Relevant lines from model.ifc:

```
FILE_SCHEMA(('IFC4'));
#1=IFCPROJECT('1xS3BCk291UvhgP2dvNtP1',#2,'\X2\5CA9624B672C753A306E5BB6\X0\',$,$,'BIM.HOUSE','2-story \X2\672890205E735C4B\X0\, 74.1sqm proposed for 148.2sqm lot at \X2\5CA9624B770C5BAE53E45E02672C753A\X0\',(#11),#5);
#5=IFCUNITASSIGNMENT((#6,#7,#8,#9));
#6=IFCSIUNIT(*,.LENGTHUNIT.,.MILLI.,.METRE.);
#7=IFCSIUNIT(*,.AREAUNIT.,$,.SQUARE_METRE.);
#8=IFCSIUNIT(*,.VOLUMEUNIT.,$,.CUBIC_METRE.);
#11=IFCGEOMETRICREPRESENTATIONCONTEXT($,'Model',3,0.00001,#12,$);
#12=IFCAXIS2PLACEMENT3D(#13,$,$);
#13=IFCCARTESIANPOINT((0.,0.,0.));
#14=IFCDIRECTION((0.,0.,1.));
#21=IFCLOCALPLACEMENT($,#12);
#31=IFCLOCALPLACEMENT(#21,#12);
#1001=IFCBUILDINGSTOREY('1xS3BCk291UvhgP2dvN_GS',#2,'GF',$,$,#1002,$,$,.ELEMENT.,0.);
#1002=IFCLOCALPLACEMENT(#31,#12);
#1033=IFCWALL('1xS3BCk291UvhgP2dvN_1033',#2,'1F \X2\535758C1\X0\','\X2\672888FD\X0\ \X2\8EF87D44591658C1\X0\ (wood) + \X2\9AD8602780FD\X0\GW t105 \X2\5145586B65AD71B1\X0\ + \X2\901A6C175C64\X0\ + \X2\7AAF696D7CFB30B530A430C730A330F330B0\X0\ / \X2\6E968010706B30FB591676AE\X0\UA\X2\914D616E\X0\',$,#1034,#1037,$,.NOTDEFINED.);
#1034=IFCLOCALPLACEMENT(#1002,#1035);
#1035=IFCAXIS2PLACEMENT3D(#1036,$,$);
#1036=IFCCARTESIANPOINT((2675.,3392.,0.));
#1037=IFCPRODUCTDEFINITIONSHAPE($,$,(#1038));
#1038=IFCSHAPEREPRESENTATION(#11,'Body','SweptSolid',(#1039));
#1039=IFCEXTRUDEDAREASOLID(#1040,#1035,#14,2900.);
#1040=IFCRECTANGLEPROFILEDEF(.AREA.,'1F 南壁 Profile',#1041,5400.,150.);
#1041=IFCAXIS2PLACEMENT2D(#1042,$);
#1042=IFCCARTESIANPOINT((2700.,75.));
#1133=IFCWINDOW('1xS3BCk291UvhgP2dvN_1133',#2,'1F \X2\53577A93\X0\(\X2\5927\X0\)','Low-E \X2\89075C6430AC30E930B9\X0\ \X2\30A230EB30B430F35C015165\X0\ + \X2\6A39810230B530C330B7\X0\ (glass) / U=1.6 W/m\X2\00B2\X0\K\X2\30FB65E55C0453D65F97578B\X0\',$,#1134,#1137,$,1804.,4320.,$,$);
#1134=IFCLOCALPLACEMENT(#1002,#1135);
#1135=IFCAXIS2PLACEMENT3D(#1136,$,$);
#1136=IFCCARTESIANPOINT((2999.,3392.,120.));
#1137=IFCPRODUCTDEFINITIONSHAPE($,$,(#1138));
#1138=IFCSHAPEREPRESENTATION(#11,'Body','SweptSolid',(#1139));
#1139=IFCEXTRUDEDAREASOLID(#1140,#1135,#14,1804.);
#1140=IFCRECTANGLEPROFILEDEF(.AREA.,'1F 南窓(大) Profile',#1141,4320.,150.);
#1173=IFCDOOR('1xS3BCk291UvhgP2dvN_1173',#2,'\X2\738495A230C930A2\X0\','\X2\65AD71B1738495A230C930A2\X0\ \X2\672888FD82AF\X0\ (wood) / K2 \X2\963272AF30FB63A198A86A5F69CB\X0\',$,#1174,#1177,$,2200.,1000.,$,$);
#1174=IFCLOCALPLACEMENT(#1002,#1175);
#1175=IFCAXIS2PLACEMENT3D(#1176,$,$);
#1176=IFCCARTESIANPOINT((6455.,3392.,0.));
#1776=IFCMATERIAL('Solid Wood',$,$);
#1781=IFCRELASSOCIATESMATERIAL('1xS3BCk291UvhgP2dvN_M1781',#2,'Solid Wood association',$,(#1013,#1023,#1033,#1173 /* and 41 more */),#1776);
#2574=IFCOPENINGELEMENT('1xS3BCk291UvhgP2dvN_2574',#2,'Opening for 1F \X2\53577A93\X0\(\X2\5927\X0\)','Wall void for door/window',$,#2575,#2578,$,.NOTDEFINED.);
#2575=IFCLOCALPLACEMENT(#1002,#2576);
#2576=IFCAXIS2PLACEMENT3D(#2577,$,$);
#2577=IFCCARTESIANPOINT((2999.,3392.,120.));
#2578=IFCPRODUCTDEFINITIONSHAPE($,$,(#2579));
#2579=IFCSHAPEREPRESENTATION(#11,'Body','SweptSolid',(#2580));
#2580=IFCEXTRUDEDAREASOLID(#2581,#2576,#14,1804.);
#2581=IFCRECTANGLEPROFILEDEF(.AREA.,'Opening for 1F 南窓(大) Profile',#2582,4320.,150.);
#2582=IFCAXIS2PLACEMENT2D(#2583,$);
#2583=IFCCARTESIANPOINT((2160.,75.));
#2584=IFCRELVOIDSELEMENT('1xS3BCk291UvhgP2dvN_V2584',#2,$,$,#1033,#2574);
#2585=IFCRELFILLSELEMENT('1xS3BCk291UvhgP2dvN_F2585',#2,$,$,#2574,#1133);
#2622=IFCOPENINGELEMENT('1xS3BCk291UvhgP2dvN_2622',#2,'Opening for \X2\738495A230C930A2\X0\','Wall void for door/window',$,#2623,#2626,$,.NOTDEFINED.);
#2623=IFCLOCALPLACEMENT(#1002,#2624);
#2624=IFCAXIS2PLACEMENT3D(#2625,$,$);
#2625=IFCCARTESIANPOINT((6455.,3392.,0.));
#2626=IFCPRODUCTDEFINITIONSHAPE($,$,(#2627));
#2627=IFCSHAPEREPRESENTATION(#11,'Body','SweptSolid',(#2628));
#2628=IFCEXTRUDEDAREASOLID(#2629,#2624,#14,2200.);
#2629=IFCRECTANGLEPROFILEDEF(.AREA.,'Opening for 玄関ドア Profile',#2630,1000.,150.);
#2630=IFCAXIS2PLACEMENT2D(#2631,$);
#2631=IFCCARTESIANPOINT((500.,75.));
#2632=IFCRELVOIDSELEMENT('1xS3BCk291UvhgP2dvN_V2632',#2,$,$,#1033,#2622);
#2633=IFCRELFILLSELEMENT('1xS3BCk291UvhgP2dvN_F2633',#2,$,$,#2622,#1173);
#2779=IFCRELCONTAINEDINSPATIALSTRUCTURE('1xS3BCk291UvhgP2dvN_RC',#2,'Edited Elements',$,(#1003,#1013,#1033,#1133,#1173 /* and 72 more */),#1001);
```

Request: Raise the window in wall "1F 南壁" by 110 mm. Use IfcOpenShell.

```python
import numpy as np
import ifcopenshell
import ifcopenshell.api.geometry
import ifcopenshell.util.placement
import ifcopenshell.util.unit

model = ifcopenshell.open("model.ifc")
unit_scale = ifcopenshell.util.unit.calculate_unit_scale(model)

window = model.by_guid("1xS3BCk291UvhgP2dvN_1133")
opening = window.FillsVoids[0].RelatingOpeningElement
dz = 110.0

shift = np.array([0.0, 0.0, dz])
# The window is not placed relative to its opening, so move both.
for product in (opening, window):
    matrix = ifcopenshell.util.placement.get_local_placement(product.ObjectPlacement)
    matrix[:3, 3] += shift
    ifcopenshell.api.geometry.edit_object_placement(model, product=product, matrix=matrix, is_si=False)

print(f"moved by {dz * unit_scale:+.3f} m")

model.write("model_v2.ifc")
```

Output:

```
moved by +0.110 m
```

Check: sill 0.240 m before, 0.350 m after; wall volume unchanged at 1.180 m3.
